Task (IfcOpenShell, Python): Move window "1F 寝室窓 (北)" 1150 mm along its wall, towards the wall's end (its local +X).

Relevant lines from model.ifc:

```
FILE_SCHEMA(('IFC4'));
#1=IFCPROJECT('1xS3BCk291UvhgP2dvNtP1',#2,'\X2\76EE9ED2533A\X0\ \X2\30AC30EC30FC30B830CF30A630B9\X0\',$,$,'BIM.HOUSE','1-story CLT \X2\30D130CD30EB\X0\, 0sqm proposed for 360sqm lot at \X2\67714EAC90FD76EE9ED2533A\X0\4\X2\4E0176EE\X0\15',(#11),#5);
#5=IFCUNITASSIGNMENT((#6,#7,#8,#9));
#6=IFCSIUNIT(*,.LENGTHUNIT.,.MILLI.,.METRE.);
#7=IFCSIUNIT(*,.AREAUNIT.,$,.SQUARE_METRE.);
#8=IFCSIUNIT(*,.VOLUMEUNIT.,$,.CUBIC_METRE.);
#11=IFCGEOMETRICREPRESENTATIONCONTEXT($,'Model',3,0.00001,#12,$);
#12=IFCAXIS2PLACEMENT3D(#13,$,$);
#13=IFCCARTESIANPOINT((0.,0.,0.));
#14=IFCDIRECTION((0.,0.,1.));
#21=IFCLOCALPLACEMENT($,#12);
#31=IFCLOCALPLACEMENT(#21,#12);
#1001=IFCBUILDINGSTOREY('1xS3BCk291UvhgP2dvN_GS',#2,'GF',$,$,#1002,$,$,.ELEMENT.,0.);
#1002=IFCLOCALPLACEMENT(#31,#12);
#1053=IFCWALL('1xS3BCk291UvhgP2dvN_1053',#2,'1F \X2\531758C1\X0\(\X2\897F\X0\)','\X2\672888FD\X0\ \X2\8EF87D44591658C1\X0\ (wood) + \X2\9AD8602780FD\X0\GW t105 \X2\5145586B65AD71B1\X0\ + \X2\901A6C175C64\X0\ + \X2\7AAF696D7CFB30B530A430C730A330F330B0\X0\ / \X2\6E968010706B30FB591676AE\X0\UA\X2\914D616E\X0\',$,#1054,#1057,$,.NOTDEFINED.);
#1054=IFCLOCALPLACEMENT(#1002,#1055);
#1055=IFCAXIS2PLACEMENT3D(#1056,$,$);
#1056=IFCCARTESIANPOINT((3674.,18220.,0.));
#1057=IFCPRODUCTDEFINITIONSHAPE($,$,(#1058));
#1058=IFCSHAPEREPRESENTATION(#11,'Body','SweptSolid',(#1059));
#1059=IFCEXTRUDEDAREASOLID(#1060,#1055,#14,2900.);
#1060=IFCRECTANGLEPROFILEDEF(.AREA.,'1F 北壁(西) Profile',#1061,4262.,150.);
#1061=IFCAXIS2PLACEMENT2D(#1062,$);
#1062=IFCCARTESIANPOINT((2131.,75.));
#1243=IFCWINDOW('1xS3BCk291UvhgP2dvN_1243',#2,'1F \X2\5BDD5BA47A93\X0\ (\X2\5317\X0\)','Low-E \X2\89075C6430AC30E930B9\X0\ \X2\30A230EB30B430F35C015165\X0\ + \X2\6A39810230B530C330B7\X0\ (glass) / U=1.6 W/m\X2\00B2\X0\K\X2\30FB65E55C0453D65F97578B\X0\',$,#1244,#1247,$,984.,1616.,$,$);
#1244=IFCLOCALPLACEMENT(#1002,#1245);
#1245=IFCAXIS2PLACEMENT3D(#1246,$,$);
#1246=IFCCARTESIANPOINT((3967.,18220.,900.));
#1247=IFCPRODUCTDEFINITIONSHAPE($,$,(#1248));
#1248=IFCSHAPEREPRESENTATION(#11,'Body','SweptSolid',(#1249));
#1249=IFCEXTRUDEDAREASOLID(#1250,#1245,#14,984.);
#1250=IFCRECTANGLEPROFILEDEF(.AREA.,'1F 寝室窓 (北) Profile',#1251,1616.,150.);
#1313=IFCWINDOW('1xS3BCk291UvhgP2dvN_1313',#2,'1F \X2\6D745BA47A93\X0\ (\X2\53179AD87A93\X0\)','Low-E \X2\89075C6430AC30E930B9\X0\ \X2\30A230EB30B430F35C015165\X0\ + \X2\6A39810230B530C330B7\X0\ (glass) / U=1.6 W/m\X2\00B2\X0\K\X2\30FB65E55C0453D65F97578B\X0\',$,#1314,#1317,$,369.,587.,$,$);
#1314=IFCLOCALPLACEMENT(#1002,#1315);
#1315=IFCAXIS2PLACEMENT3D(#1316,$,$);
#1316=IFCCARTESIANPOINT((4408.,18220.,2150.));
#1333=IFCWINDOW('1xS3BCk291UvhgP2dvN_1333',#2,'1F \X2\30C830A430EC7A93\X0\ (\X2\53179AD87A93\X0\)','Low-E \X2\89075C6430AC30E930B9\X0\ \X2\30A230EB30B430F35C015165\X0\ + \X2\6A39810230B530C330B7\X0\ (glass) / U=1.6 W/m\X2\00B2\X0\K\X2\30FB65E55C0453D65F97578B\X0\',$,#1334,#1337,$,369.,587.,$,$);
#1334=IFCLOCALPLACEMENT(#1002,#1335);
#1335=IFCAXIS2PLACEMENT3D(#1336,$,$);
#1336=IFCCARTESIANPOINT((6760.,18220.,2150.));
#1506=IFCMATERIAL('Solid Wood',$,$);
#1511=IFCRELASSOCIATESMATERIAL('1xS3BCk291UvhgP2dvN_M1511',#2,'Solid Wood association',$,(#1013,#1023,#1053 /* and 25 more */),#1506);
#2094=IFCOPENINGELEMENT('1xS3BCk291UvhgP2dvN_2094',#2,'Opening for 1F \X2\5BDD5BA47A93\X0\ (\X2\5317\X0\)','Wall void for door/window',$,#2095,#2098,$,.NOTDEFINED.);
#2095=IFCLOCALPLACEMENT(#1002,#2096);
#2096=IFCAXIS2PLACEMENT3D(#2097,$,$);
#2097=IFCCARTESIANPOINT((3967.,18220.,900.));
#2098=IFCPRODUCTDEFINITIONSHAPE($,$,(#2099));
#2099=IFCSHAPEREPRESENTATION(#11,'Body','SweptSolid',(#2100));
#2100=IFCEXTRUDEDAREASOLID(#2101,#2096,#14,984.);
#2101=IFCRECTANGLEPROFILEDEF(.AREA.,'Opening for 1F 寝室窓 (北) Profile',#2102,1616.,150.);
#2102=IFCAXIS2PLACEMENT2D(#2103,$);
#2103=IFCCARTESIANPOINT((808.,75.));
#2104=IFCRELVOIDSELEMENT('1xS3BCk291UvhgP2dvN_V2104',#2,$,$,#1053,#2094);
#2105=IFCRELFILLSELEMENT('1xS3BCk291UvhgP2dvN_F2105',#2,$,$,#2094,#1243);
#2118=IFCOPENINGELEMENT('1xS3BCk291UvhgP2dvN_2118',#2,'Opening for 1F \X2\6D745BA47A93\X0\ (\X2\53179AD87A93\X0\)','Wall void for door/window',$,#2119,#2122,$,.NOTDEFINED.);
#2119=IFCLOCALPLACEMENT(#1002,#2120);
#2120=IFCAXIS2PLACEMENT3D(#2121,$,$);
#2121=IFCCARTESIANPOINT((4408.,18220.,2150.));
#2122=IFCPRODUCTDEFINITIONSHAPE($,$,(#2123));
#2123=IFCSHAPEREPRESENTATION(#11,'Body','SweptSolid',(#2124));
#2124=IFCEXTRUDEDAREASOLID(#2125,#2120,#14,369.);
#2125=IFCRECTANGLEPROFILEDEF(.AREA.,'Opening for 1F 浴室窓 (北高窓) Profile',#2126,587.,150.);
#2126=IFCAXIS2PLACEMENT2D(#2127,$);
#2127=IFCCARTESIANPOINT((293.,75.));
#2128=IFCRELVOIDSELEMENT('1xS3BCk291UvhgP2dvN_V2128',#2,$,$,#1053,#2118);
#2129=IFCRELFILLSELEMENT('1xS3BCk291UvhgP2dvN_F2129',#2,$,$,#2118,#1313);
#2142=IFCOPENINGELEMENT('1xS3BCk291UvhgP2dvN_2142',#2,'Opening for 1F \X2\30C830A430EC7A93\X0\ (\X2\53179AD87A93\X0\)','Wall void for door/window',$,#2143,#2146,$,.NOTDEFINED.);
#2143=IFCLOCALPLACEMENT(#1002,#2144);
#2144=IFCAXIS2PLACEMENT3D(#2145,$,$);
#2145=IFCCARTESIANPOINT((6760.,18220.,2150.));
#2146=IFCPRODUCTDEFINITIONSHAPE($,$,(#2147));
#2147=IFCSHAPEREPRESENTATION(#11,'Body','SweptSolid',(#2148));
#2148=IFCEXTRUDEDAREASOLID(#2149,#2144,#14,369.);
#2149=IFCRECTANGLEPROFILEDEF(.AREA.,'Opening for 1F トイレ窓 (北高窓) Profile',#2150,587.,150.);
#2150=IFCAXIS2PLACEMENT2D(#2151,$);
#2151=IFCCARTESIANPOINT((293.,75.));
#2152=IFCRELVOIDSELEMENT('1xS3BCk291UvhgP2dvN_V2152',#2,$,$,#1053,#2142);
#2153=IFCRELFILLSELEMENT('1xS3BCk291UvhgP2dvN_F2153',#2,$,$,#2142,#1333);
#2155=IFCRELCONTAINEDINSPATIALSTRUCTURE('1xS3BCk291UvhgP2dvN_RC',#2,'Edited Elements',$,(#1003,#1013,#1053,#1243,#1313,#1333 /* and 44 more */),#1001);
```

```python
import ifcopenshell
import ifcopenshell.api.geometry
import ifcopenshell.util.placement
import ifcopenshell.util.unit

model = ifcopenshell.open("model.ifc")
unit_scale = ifcopenshell.util.unit.calculate_unit_scale(model)

window = model.by_guid("1xS3BCk291UvhgP2dvN_1243")
opening = window.FillsVoids[0].RelatingOpeningElement
wall = opening.VoidsElements[0].RelatingBuildingElement

wall_matrix = ifcopenshell.util.placement.get_local_placement(wall.ObjectPlacement)
shift = wall_matrix[:3, 0] * 1.15 / unit_scale
before = ifcopenshell.util.placement.get_local_placement(window.ObjectPlacement)[:3, 3].copy()

# The window is not placed relative to its opening, so move both.
for product in (opening, window):
    matrix = ifcopenshell.util.placement.get_local_placement(product.ObjectPlacement)
    matrix[:3, 3] += shift
    ifcopenshell.api.geometry.edit_object_placement(model, product=product, matrix=matrix, is_si=False)

after = ifcopenshell.util.placement.get_local_placement(window.ObjectPlacement)[:3, 3]
print("window moved by", (after - before).round(3) + 0.0)

model.write("model-out.ifc")
```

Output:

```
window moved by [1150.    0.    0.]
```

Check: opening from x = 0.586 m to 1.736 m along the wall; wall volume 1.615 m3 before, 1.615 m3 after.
